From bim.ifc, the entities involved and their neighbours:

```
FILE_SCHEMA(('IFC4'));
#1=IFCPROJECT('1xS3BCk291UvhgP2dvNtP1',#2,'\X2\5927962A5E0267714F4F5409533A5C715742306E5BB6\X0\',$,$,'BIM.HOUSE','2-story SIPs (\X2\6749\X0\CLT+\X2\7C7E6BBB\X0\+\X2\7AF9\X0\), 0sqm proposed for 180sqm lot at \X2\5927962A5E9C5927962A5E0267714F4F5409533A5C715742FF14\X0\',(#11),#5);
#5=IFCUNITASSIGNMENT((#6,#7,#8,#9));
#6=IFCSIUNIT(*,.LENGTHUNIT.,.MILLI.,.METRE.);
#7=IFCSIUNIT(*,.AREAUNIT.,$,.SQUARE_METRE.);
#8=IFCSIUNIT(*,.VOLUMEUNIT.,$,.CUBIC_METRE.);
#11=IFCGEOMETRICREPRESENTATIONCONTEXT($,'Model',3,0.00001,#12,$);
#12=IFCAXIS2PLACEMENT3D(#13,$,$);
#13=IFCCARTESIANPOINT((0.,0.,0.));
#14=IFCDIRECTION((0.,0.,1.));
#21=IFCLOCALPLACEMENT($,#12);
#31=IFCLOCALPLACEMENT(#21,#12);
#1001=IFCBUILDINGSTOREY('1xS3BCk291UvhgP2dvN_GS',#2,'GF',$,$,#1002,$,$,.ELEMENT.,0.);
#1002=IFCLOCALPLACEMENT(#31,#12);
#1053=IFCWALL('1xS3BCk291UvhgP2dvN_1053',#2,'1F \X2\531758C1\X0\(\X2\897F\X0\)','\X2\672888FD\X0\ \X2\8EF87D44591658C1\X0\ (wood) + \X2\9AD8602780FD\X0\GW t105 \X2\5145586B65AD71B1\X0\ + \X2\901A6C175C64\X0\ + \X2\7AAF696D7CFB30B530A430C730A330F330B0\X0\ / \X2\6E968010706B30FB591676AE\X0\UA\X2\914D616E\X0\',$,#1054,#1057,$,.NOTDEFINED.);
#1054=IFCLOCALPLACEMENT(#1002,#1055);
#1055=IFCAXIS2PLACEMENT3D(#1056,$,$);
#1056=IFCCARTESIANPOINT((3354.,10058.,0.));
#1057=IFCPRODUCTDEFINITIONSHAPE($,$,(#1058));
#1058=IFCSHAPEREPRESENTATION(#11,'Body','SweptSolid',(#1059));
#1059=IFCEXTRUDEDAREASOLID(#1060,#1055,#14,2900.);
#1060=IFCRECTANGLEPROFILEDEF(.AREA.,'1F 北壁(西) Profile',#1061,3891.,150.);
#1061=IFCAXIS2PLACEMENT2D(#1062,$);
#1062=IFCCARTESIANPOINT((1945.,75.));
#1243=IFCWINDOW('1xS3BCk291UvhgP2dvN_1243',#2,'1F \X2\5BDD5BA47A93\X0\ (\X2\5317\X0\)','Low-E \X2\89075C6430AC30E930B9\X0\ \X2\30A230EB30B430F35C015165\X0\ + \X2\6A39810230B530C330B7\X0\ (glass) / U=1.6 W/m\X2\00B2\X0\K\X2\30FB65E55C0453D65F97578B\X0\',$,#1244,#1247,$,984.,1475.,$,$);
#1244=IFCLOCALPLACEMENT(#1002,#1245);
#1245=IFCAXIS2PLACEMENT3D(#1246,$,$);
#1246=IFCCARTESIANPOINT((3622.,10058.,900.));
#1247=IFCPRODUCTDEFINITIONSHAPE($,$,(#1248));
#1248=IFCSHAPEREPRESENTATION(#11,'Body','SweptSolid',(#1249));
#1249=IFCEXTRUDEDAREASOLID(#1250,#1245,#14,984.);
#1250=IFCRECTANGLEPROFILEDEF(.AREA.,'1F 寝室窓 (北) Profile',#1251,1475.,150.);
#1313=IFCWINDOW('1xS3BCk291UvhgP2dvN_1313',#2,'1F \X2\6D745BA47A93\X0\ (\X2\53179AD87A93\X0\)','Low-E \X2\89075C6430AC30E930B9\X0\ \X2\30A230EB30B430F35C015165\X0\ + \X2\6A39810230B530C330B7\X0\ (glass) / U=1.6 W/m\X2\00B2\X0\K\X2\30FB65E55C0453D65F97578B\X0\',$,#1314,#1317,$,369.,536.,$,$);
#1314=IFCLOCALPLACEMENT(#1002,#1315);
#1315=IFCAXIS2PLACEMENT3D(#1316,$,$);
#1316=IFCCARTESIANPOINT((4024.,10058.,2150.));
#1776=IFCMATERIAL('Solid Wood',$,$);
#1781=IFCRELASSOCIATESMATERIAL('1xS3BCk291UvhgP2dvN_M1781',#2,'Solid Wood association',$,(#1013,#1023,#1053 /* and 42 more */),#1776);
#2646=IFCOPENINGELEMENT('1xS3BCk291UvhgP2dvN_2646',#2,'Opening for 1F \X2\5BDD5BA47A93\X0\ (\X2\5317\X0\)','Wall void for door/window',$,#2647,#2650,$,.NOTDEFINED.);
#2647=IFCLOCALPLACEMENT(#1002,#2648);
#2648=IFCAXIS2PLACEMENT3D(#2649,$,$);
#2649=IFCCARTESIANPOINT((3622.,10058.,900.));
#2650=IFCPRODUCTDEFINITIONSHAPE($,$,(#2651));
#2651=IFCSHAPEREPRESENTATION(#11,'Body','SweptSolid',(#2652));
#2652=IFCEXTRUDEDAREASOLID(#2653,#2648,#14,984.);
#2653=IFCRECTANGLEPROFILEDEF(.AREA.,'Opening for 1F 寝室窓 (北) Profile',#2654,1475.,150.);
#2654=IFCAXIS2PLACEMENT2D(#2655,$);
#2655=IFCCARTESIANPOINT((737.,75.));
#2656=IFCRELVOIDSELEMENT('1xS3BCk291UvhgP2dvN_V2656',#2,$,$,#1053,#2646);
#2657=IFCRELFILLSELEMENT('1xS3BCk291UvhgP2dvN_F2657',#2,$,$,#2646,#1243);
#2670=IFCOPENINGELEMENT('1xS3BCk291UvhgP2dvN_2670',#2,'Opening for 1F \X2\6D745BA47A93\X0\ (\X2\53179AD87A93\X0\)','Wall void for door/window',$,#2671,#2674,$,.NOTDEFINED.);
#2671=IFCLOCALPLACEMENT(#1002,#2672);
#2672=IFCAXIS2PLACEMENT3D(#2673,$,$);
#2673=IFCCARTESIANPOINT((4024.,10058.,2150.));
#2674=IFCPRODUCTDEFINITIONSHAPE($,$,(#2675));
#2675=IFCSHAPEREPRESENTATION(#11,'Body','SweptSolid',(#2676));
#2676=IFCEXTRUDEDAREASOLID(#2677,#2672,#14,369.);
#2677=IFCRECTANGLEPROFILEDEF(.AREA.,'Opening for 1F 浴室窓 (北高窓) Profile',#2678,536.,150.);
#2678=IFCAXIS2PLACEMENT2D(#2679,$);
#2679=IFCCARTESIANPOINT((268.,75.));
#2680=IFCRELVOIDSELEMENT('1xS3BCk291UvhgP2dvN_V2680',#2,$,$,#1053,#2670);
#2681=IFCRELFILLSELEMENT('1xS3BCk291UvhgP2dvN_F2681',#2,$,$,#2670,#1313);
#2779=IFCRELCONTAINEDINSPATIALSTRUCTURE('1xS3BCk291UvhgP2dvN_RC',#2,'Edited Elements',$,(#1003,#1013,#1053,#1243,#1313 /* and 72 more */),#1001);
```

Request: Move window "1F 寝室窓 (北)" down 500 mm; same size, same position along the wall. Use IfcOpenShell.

```python
import numpy as np
import ifcopenshell
import ifcopenshell.api.geometry
import ifcopenshell.util.placement
import ifcopenshell.util.unit

model = ifcopenshell.open("bim.ifc")
unit_scale = ifcopenshell.util.unit.calculate_unit_scale(model)

window = model.by_guid("1xS3BCk291UvhgP2dvN_1243")
opening = window.FillsVoids[0].RelatingOpeningElement
dz = -0.5 / unit_scale

shift = np.array([0.0, 0.0, dz])
# The window is not placed relative to its opening, so move both.
for product in (opening, window):
    matrix = ifcopenshell.util.placement.get_local_placement(product.ObjectPlacement)
    matrix[:3, 3] += shift
    ifcopenshell.api.geometry.edit_object_placement(model, product=product, matrix=matrix, is_si=False)

print(f"moved by {dz * unit_scale:+.3f} m")

model.write("bim_v2.ifc")
```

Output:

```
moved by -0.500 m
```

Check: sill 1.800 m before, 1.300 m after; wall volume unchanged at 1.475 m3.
